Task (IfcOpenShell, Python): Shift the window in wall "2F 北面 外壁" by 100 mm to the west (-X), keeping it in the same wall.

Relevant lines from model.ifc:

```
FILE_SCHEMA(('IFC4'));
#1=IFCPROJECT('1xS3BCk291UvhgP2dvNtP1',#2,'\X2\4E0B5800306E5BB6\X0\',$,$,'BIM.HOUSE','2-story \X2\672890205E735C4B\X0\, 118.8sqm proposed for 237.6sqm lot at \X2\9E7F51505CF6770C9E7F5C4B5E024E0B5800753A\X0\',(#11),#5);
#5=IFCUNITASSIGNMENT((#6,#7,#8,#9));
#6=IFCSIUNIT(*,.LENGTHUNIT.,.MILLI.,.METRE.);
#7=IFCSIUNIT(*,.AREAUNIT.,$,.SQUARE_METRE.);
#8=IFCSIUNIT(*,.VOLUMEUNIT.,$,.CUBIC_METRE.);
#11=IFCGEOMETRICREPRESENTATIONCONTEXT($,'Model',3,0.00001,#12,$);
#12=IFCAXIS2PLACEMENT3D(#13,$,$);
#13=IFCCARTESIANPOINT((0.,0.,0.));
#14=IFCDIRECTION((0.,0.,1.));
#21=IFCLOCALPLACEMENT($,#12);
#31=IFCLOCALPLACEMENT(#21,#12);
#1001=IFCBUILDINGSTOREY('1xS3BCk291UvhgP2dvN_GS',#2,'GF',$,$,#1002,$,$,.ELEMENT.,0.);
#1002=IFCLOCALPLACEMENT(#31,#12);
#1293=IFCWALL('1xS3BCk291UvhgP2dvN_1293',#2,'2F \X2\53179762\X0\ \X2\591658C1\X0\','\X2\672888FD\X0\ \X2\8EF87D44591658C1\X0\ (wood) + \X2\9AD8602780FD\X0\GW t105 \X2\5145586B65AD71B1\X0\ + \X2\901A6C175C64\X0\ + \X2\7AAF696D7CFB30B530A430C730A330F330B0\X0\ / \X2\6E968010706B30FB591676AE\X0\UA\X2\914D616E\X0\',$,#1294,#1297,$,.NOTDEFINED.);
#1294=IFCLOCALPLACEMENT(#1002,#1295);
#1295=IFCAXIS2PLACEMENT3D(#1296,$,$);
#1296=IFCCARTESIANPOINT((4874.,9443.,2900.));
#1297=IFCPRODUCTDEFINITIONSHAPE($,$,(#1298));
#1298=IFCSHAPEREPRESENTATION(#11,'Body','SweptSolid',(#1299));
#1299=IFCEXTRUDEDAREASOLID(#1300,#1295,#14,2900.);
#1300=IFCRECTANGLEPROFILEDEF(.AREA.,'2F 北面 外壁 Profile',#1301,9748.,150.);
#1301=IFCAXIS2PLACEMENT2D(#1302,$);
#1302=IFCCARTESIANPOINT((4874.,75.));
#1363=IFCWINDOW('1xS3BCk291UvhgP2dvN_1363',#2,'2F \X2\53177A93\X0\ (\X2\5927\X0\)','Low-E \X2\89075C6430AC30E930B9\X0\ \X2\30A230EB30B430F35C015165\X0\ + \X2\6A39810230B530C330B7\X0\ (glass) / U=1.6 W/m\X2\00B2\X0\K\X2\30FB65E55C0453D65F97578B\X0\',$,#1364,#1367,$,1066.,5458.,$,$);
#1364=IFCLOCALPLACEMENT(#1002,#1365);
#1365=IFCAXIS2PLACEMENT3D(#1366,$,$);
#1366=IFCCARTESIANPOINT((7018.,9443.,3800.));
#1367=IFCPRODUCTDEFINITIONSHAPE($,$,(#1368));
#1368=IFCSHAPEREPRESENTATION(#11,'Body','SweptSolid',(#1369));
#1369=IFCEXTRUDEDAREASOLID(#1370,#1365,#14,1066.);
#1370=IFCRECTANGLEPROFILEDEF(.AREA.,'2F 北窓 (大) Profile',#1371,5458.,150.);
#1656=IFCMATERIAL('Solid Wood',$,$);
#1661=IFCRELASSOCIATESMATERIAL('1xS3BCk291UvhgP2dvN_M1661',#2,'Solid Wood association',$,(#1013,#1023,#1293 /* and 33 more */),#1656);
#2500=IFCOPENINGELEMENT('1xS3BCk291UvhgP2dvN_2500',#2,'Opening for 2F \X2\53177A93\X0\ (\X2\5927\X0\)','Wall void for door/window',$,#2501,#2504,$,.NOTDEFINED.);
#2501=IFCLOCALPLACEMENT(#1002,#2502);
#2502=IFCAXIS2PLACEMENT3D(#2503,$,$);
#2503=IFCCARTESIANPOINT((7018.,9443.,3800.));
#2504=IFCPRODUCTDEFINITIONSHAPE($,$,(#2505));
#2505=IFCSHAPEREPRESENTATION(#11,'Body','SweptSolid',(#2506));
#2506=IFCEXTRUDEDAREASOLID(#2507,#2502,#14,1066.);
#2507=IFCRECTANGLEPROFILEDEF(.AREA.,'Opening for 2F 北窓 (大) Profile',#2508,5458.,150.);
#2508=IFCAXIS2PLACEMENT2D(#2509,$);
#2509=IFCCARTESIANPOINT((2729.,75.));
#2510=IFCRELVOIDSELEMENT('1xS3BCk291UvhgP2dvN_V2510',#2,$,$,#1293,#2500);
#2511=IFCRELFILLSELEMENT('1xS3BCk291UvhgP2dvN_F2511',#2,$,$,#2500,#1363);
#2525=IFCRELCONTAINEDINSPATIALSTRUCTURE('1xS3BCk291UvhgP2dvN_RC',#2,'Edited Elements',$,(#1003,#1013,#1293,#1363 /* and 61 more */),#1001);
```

```python
import ifcopenshell
import ifcopenshell.api.geometry
import ifcopenshell.util.placement

model = ifcopenshell.open("model.ifc")

window = model.by_guid("1xS3BCk291UvhgP2dvN_1363")
opening = window.FillsVoids[0].RelatingOpeningElement
wall = opening.VoidsElements[0].RelatingBuildingElement

wall_matrix = ifcopenshell.util.placement.get_local_placement(wall.ObjectPlacement)
shift = wall_matrix[:3, 0] * -100.0
before = ifcopenshell.util.placement.get_local_placement(window.ObjectPlacement)[:3, 3].copy()

# The window is not placed relative to its opening, so move both.
for product in (opening, window):
    matrix = ifcopenshell.util.placement.get_local_placement(product.ObjectPlacement)
    matrix[:3, 3] += shift
    ifcopenshell.api.geometry.edit_object_placement(model, product=product, matrix=matrix, is_si=False)

after = ifcopenshell.util.placement.get_local_placement(window.ObjectPlacement)[:3, 3]
print("window moved by", (after - before).round(3) + 0.0)

model.write("model_edited.ifc")
```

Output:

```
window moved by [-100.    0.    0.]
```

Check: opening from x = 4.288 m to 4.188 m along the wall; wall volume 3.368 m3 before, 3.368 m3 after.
